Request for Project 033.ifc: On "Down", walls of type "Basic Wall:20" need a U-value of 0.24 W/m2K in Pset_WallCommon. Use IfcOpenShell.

First a look at what the model holds.

```python
import ifcopenshell
import ifcopenshell.util.element

model = ifcopenshell.open("Project 033.ifc")
print(model.schema)
storey = next(s for s in model.by_type("IfcBuildingStorey") if s.Name == "Down")
walls = [e for e in ifcopenshell.util.element.get_decomposition(storey) if e.is_a("IfcWall")]
seen = {}
for e in walls:
    element_type = ifcopenshell.util.element.get_type(e)
    key = (element_type.Name if element_type != e and element_type else None, ifcopenshell.util.element.get_pset(e, "Pset_WallCommon", "ThermalTransmittance"))
    seen[key] = seen.get(key, 0) + 1
for (name, value), count in sorted(seen.items(), key=str):
    print(count, "x", name, "|", value)
```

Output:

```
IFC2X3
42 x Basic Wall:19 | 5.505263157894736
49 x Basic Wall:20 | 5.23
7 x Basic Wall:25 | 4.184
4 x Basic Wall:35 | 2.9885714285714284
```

```python
import ifcopenshell
import ifcopenshell.api.pset
import ifcopenshell.util.element

model = ifcopenshell.open("Project 033.ifc")

storey = next(s for s in model.by_type("IfcBuildingStorey") if s.Name == "Down")
walls = [e for e in ifcopenshell.util.element.get_decomposition(storey) if e.is_a("IfcWall")]

count = 0
for e in walls:
    element_type = ifcopenshell.util.element.get_type(e)
    if element_type in (None, e) or element_type.Name != "Basic Wall:20":
        continue
    # add_pset returns the element's existing set when there is one.
    pset = ifcopenshell.api.pset.add_pset(model, product=e, name="Pset_WallCommon")
    ifcopenshell.api.pset.edit_pset(model, pset=pset, properties={"ThermalTransmittance": 0.24})
    count += 1

print(count, "walls updated")

model.write("Project 033-out.ifc")
```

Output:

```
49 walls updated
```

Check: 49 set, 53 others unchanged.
